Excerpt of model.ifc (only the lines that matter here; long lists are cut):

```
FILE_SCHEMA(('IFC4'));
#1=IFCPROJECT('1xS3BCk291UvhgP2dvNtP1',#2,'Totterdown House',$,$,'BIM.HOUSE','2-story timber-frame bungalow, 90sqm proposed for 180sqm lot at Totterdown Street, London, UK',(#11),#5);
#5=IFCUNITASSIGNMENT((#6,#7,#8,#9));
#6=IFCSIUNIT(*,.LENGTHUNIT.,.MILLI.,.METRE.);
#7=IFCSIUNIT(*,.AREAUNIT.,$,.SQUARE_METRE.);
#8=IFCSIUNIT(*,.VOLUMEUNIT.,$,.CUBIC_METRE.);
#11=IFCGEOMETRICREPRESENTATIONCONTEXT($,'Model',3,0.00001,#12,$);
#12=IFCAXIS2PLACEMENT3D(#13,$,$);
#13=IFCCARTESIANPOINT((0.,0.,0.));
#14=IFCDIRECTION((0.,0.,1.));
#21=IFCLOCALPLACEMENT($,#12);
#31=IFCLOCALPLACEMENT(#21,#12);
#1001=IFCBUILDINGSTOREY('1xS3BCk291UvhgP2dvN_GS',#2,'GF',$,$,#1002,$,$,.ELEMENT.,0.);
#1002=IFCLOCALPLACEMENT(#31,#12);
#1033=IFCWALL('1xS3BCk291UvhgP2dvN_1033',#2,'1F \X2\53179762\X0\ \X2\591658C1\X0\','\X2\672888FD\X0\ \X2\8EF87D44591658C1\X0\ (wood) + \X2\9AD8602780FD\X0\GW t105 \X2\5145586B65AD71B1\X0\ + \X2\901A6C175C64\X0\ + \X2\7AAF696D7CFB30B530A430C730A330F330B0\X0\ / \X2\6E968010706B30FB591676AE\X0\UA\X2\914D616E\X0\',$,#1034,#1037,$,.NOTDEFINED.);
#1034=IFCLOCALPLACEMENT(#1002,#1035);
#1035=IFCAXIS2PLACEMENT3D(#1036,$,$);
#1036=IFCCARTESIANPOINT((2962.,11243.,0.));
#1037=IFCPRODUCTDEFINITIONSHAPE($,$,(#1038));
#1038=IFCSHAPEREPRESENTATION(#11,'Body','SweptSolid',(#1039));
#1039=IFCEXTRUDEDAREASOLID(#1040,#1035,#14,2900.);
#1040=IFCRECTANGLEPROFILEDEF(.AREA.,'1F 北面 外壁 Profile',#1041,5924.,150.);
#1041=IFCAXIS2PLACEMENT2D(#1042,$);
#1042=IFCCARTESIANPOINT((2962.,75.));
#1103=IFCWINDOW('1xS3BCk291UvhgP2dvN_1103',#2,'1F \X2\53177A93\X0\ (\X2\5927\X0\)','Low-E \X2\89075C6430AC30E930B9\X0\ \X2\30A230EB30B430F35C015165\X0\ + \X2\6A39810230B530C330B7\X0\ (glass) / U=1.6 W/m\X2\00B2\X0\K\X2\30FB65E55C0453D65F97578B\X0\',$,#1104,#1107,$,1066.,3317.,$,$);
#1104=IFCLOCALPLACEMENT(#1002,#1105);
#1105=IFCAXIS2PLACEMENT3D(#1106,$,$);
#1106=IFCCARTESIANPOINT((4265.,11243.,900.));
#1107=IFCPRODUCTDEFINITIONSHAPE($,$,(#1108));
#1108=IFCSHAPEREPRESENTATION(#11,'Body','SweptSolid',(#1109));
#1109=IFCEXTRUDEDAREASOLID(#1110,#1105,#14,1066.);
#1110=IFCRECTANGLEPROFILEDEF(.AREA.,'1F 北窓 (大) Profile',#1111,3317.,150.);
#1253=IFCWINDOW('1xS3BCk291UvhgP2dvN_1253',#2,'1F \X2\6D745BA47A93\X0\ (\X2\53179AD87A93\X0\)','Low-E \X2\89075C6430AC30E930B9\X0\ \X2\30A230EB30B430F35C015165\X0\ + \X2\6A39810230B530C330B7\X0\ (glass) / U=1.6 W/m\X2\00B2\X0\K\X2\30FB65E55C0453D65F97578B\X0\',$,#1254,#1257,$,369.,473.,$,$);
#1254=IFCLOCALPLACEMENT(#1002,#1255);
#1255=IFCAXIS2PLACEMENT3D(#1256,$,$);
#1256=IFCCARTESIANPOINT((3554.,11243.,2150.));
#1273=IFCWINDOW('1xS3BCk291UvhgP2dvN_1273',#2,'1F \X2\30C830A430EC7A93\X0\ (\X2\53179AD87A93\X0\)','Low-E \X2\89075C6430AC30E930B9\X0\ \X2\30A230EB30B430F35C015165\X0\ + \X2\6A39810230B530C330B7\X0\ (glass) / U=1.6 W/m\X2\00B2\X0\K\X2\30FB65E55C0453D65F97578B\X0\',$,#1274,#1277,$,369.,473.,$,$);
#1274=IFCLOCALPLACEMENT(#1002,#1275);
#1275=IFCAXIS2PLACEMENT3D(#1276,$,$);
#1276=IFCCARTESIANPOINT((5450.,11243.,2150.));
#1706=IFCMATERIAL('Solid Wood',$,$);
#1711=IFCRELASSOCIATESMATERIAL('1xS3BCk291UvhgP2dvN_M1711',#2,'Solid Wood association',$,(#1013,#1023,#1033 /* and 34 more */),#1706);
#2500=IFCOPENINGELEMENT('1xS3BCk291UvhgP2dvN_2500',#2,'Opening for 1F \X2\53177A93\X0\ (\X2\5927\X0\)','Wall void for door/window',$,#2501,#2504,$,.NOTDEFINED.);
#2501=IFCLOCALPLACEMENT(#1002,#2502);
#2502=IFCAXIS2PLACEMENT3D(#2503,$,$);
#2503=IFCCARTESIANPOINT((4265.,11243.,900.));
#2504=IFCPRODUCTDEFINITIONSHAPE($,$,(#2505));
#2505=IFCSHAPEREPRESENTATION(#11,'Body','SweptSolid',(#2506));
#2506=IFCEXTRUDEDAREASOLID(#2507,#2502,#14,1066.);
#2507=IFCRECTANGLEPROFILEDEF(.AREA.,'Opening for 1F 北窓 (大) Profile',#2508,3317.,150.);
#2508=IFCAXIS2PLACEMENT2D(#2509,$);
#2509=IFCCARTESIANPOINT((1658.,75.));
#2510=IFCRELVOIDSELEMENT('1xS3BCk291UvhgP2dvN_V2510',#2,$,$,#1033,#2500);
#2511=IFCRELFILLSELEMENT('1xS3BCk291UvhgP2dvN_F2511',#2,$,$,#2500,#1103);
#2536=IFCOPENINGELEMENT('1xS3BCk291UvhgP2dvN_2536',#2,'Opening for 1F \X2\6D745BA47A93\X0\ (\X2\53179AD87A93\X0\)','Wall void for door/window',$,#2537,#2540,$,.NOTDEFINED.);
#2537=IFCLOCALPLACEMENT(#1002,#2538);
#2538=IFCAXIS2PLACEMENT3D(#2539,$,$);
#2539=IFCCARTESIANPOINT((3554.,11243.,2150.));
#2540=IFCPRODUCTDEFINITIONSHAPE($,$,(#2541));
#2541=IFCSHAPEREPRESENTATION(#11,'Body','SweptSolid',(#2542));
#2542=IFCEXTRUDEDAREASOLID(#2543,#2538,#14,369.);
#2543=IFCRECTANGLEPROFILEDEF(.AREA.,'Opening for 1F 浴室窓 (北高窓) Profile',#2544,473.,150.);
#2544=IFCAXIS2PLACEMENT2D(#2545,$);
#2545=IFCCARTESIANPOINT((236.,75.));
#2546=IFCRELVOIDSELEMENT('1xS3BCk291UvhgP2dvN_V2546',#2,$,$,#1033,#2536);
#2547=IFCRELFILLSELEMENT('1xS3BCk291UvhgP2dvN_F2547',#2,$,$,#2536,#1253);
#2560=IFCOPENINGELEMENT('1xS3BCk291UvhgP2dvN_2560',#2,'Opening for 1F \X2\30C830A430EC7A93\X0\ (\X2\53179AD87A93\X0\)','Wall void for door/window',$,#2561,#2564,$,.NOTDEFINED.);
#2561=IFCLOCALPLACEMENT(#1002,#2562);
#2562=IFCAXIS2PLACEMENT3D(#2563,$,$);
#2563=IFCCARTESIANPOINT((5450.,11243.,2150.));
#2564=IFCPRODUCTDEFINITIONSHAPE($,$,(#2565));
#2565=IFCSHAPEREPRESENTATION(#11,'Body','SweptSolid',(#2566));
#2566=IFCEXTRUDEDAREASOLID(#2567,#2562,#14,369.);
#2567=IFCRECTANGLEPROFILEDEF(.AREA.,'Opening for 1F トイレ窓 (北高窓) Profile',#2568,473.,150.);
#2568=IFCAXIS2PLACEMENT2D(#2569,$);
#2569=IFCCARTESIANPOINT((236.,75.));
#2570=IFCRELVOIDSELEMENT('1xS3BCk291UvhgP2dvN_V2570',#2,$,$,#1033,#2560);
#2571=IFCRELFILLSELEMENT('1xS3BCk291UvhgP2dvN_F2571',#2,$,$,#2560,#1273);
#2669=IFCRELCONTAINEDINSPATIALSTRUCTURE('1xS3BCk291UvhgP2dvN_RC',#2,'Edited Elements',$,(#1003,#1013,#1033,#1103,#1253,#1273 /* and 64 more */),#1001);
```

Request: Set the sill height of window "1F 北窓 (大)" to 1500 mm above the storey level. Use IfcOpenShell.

```python
import numpy as np
import ifcopenshell
import ifcopenshell.api.geometry
import ifcopenshell.geom
import ifcopenshell.util.element
import ifcopenshell.util.placement
import ifcopenshell.util.shape
import ifcopenshell.util.unit

model = ifcopenshell.open("model.ifc")
unit_scale = ifcopenshell.util.unit.calculate_unit_scale(model)

window = model.by_guid("1xS3BCk291UvhgP2dvN_1103")
opening = window.FillsVoids[0].RelatingOpeningElement
storey = ifcopenshell.util.element.get_container(window, ifc_class="IfcBuildingStorey")
level = ifcopenshell.util.placement.get_local_placement(storey.ObjectPlacement)[2, 3]

# The opening's origin need not be at the sill, so measure its lowest point.
shape = ifcopenshell.geom.create_shape(ifcopenshell.geom.settings(), opening)
bottom = ifcopenshell.util.shape.get_shape_bottom_elevation(shape, shape.geometry) / unit_scale
dz = level + 1500.0 - bottom

shift = np.array([0.0, 0.0, dz])
# The window is not placed relative to its opening, so move both.
for product in (opening, window):
    matrix = ifcopenshell.util.placement.get_local_placement(product.ObjectPlacement)
    matrix[:3, 3] += shift
    ifcopenshell.api.geometry.edit_object_placement(model, product=product, matrix=matrix, is_si=False)

print(f"moved by {dz * unit_scale:+.3f} m")

model.write("model_updated.ifc")
```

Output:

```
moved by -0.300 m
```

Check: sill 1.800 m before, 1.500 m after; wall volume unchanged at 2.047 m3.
